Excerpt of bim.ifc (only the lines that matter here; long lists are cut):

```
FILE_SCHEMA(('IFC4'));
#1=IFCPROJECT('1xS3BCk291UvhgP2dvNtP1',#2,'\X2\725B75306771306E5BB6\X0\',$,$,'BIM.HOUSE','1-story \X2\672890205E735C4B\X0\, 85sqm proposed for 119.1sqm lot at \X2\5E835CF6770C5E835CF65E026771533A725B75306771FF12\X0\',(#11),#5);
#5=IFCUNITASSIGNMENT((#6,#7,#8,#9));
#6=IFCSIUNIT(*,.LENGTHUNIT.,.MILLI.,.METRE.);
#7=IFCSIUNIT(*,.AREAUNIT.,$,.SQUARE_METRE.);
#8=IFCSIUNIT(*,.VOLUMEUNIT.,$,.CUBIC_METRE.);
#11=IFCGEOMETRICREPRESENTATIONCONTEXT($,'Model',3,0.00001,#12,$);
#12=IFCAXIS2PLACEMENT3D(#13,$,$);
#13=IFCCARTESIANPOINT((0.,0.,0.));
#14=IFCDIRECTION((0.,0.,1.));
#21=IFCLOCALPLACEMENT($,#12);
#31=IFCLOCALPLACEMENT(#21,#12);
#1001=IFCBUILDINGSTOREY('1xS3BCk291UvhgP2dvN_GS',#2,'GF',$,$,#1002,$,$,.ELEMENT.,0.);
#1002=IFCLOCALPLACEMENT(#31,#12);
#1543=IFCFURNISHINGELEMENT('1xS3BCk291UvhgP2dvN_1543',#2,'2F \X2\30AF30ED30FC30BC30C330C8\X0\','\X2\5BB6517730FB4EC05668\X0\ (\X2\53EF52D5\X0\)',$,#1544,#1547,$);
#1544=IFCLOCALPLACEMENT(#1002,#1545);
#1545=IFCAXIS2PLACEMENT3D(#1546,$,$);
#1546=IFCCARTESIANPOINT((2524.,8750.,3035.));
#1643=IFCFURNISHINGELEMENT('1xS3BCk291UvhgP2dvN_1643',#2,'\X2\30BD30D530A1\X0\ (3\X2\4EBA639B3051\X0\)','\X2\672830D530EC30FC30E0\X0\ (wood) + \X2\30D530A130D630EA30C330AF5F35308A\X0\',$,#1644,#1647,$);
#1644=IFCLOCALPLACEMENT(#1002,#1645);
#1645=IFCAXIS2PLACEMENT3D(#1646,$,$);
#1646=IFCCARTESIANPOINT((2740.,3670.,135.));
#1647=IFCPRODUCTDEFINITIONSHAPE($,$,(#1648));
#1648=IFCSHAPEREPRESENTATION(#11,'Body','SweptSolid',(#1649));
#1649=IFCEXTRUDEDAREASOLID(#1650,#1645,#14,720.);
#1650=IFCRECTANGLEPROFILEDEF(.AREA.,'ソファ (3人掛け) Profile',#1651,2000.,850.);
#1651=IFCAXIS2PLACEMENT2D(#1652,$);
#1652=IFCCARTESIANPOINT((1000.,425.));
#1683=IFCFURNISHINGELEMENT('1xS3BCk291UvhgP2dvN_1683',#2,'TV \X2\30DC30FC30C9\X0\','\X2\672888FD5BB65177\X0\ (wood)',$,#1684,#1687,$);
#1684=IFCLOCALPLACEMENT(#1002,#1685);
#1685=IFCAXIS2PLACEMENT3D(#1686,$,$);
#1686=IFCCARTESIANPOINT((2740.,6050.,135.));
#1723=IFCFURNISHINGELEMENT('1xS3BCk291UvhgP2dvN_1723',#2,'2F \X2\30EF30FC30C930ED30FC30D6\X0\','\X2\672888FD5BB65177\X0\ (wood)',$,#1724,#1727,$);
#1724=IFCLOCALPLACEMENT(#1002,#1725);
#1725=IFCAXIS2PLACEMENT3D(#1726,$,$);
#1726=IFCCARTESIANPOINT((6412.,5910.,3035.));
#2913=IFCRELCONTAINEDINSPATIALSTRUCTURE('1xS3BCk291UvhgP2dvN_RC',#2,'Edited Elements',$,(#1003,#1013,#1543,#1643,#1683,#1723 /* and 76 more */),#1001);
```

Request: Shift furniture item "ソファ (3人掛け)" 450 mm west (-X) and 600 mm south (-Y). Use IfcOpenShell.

```python
import ifcopenshell
import ifcopenshell.api.geometry
import ifcopenshell.util.placement
import ifcopenshell.util.unit

model = ifcopenshell.open("bim.ifc")
unit_scale = ifcopenshell.util.unit.calculate_unit_scale(model)

item = model.by_guid("1xS3BCk291UvhgP2dvN_1643")
matrix = ifcopenshell.util.placement.get_local_placement(item.ObjectPlacement)
matrix[0, 3] -= 0.45 / unit_scale
matrix[1, 3] -= 0.6 / unit_scale
ifcopenshell.api.geometry.edit_object_placement(model, product=item, matrix=matrix, is_si=False)

print(ifcopenshell.util.placement.get_local_placement(item.ObjectPlacement).round(3) + 0.0)

model.write("bim_edited.ifc")
```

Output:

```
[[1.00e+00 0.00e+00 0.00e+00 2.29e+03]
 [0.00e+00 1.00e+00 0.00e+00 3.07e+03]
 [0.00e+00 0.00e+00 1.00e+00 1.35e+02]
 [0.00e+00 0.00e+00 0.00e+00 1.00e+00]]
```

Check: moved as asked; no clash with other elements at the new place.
